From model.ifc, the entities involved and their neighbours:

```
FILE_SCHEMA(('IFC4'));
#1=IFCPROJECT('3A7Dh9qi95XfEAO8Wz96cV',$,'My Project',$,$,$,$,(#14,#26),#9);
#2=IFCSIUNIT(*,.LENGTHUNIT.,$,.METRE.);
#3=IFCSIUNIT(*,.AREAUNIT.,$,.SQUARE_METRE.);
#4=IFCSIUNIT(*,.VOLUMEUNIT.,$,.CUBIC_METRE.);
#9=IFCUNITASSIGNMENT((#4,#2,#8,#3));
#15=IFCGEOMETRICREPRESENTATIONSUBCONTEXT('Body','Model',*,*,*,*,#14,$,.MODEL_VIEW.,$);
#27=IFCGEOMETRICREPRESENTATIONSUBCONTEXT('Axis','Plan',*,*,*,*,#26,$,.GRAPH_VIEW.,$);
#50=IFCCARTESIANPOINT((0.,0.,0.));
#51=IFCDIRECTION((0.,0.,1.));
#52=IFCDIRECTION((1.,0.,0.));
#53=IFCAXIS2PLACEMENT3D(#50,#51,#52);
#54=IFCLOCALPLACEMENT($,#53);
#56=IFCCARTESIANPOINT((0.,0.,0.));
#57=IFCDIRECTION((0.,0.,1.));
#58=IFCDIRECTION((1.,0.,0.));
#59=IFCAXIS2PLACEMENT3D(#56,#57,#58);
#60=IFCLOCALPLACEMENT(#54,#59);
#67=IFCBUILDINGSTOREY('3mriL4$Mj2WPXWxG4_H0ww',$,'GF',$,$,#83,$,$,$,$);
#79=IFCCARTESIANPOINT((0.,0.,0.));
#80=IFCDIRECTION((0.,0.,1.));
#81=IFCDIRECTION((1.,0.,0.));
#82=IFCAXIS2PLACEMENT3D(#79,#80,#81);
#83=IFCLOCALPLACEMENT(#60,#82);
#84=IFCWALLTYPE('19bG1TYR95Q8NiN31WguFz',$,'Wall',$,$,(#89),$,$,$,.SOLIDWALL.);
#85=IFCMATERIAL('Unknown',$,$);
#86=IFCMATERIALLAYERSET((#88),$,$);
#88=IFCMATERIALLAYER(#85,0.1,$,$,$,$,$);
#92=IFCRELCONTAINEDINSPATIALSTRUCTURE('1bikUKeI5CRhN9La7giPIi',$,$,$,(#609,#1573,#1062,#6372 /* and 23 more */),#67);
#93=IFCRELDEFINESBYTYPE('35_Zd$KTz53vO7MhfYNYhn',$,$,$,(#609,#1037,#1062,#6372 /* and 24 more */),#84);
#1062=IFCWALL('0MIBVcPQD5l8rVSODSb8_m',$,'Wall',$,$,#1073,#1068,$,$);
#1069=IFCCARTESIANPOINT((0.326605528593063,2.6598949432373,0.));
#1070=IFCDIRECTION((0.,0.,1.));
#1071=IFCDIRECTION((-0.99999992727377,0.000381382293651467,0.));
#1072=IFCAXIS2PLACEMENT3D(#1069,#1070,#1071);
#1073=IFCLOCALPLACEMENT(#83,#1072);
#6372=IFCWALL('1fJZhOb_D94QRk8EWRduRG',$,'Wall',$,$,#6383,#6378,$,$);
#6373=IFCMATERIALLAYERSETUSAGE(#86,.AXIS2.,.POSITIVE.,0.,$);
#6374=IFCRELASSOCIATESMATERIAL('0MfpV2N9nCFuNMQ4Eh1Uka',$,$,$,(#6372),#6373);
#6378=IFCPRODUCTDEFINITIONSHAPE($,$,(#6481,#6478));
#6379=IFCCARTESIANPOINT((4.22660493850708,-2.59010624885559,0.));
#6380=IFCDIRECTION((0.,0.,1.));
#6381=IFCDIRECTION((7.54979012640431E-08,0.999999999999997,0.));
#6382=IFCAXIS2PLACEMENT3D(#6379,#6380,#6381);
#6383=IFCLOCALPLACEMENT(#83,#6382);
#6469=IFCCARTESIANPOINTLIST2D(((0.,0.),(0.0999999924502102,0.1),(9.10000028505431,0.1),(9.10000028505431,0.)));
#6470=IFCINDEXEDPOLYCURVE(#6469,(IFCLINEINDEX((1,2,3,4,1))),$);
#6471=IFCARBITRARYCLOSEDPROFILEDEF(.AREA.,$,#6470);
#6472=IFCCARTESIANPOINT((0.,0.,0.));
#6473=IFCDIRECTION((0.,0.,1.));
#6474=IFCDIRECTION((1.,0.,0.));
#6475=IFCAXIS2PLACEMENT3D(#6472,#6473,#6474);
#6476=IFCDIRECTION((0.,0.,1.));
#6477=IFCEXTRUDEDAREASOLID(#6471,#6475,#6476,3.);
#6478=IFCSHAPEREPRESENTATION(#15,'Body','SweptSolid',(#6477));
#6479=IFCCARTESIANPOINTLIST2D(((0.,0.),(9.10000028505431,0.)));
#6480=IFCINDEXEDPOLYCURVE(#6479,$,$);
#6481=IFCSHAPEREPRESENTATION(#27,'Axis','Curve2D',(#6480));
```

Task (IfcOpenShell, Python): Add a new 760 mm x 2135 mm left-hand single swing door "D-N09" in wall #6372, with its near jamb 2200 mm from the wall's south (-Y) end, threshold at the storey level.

```python
import numpy as np
import ifcopenshell
import ifcopenshell.api.feature
import ifcopenshell.api.geometry
import ifcopenshell.api.root
import ifcopenshell.api.spatial
import ifcopenshell.geom
import ifcopenshell.util.element
import ifcopenshell.util.placement
import ifcopenshell.util.representation
import ifcopenshell.util.shape
import ifcopenshell.util.unit

model = ifcopenshell.open("model.ifc")
unit_scale = ifcopenshell.util.unit.calculate_unit_scale(model)
settings = ifcopenshell.geom.settings()


def volume(element):
    """Net volume in cubic metres, openings subtracted."""
    shape = ifcopenshell.geom.create_shape(settings, element)
    return ifcopenshell.util.shape.get_volume(shape.geometry)


wall = model.by_id(6372)
storey = ifcopenshell.util.element.get_container(wall, ifc_class="IfcBuildingStorey")
context = ifcopenshell.util.representation.get_context(model, "Model", "Body", "MODEL_VIEW")
before = volume(wall)

width, height, from_end, sill = 0.76, 2.135, 2.2, 0.0  # metres

# The wall runs along its own X axis, and the end named is its -X end.
wall_shape = ifcopenshell.geom.create_shape(settings, wall)
x, y, z = ifcopenshell.util.shape.get_vertices(wall_shape.geometry).T
start = x.min() + from_end
face, thickness = float(y.min()), float(y.max() - y.min())
wall_matrix = ifcopenshell.util.placement.get_local_placement(wall.ObjectPlacement)
level = ifcopenshell.util.placement.get_local_placement(storey.ObjectPlacement)[2, 3]


def in_wall(x, y):
    """Placement at x, y metres in the wall's axes, at sill height."""
    matrix = wall_matrix.copy()
    matrix[:, 3] = wall_matrix @ np.array([x / unit_scale, y / unit_scale, 0.0, 1.0])
    matrix[2, 3] = level + sill / unit_scale
    return matrix


# Opening: a box that overshoots both wall faces by 50 mm.
opening = ifcopenshell.api.root.create_entity(model, ifc_class="IfcOpeningElement", predefined_type="OPENING")
box = ifcopenshell.api.geometry.add_wall_representation(
    model, context=context, length=width, height=height, thickness=thickness + 0.1
)
ifcopenshell.api.geometry.assign_representation(model, product=opening, representation=box)
ifcopenshell.api.geometry.edit_object_placement(model, product=opening, matrix=in_wall(start, face - 0.05), is_si=False)
ifcopenshell.api.feature.add_feature(model, feature=opening, element=wall)

door = ifcopenshell.api.root.create_entity(model, ifc_class="IfcDoor", name="D-N09", predefined_type="DOOR")
door.OverallWidth, door.OverallHeight = width / unit_scale, height / unit_scale
door.OperationType = "SINGLE_SWING_LEFT"
body = ifcopenshell.api.geometry.add_door_representation(
    model,
    context=context,
    overall_width=door.OverallWidth,
    overall_height=door.OverallHeight,
    operation_type="SINGLE_SWING_LEFT",
    lining_properties={"LiningDepth": thickness / unit_scale, "ThresholdDepth": thickness / unit_scale},
)
ifcopenshell.api.geometry.assign_representation(model, product=door, representation=body)
ifcopenshell.api.spatial.assign_container(model, products=[door], relating_structure=storey)
ifcopenshell.api.feature.add_filling(model, opening=opening, element=door)

# The lining spans the wall, so the door starts at the wall face.
ifcopenshell.api.geometry.edit_object_placement(model, product=door, matrix=in_wall(start, face), is_si=False)

after = volume(wall)

print(f"wall volume {before:.3f} -> {after:.3f} m3")

model.write("model_rev.ifc")
```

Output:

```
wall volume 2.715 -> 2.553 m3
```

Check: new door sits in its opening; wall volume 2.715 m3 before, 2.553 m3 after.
